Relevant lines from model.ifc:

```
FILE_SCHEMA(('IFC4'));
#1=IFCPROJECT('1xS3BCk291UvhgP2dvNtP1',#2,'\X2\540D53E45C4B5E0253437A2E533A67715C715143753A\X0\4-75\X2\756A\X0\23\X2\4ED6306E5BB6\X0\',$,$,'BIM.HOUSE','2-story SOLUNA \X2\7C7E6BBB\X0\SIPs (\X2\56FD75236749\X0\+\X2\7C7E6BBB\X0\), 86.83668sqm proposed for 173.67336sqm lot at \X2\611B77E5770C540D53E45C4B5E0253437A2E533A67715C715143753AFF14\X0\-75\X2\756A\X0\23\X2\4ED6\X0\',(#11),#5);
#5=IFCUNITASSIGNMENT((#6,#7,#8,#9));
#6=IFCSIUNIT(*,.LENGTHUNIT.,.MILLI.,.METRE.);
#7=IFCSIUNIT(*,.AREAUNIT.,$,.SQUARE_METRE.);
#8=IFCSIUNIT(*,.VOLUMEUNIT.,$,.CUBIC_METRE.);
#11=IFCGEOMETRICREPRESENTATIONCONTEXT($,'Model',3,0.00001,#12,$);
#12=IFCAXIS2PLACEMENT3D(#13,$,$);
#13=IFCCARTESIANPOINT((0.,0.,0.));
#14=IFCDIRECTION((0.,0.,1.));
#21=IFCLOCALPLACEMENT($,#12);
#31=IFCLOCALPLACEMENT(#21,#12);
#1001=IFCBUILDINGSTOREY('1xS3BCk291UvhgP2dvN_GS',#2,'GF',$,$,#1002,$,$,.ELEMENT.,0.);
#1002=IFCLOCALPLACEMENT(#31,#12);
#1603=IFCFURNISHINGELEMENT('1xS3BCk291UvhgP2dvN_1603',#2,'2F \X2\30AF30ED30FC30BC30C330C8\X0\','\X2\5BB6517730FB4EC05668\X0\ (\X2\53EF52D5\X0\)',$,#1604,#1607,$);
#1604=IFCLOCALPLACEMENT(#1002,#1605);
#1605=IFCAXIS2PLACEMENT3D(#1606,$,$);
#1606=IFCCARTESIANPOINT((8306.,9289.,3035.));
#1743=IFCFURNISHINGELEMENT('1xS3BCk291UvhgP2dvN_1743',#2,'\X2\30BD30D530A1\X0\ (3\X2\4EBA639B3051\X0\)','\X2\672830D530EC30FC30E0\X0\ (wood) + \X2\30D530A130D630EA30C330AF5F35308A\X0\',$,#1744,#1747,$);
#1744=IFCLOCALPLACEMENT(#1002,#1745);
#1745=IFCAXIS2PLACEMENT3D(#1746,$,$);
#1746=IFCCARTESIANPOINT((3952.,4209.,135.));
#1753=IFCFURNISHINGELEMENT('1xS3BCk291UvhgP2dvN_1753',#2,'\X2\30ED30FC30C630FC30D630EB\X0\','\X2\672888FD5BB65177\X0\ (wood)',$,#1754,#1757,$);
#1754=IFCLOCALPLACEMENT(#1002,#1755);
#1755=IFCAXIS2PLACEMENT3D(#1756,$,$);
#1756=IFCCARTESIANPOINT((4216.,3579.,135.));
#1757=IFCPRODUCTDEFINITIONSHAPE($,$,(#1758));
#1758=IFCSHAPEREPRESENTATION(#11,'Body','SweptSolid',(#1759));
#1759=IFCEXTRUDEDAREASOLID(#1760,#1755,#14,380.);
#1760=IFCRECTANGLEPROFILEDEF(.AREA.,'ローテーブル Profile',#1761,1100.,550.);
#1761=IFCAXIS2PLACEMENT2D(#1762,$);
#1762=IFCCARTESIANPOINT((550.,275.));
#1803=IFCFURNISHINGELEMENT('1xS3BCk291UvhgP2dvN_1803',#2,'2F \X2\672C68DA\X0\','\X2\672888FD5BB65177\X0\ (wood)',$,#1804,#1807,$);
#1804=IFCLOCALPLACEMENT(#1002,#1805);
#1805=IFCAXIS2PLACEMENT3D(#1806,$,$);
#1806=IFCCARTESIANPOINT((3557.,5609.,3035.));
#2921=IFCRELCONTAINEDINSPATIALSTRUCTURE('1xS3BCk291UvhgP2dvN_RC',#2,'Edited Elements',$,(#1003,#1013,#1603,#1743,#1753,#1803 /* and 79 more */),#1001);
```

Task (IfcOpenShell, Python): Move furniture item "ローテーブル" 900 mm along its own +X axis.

```python
import ifcopenshell
import ifcopenshell.api.geometry
import ifcopenshell.util.placement
import ifcopenshell.util.unit

model = ifcopenshell.open("model.ifc")
unit_scale = ifcopenshell.util.unit.calculate_unit_scale(model)

item = model.by_id(1753)
matrix = ifcopenshell.util.placement.get_local_placement(item.ObjectPlacement)
matrix[:3, 3] += matrix[:3, 0] * 0.9 / unit_scale
ifcopenshell.api.geometry.edit_object_placement(model, product=item, matrix=matrix, is_si=False)

print(ifcopenshell.util.placement.get_local_placement(item.ObjectPlacement).round(3) + 0.0)

model.write("model_edited.ifc")
```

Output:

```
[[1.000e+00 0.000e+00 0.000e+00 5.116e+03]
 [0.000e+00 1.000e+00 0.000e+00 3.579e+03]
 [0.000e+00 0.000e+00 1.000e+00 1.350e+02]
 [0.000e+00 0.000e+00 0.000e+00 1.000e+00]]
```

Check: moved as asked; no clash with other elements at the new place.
